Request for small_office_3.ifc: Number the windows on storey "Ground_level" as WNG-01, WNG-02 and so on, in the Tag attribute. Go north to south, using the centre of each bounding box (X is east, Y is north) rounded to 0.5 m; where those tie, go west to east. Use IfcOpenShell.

First a look at what the model holds.

```python
import ifcopenshell
import ifcopenshell.util.element
import ifcopenshell.util.placement

model = ifcopenshell.open("small_office_3.ifc")
print(model.schema)
storey = next(s for s in model.by_type("IfcBuildingStorey") if s.Name == "Ground_level")
windows = [e for e in ifcopenshell.util.element.get_decomposition(storey) if e.is_a("IfcWindow")]
for e in sorted(windows, key=lambda e: e.id()):
    origin = ifcopenshell.util.placement.get_local_placement(e.ObjectPlacement)[:3, 3]
    print(e.id(), e.Tag, e.Name, origin.round(2) + 0.0, sep=" | ")
```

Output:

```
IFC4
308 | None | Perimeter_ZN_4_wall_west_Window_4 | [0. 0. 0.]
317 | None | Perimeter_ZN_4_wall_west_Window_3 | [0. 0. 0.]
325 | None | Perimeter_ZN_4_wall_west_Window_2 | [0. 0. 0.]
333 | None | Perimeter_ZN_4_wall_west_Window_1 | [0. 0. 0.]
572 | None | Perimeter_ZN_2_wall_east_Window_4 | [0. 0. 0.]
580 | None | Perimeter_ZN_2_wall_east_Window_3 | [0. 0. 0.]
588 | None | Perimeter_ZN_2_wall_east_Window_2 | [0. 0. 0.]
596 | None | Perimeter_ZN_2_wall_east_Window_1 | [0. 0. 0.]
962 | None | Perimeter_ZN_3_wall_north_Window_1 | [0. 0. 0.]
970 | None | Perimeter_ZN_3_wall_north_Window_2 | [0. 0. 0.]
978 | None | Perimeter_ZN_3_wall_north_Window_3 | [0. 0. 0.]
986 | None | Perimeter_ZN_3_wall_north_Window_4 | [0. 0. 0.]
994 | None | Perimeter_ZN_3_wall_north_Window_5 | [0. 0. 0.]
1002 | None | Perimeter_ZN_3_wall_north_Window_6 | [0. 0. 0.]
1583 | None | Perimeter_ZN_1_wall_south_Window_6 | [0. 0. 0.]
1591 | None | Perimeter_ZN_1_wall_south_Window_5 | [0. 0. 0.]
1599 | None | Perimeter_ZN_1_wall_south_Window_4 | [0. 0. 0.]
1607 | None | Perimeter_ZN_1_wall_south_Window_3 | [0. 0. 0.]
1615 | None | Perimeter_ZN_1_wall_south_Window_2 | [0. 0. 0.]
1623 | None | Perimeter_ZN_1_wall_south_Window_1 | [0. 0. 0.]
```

```python
import ifcopenshell
import ifcopenshell.geom
import ifcopenshell.util.element
import ifcopenshell.util.shape

model = ifcopenshell.open("small_office_3.ifc")
settings = ifcopenshell.geom.settings()
settings.set("use-world-coords", True)


def centre(element):
    shape = ifcopenshell.geom.create_shape(settings, element)
    return ifcopenshell.util.shape.get_bbox_centroid(shape.geometry)


storey = next(s for s in model.by_type("IfcBuildingStorey") if s.Name == "Ground_level")
windows = [e for e in ifcopenshell.util.element.get_decomposition(storey) if e.is_a("IfcWindow")]

# Insertion points can sit at a corner or the storey origin, so sort by the geometry (in metres).
centres = {e: centre(e) for e in windows}
windows.sort(key=lambda e: (-round(centres[e][1] / 0.5), centres[e][0]))

for i, e in enumerate(windows, start=1):
    number = f"WNG-{i:02d}"
    e.Tag = number
    print(e.id(), number)

model.write("small_office_3_edited.ifc")
```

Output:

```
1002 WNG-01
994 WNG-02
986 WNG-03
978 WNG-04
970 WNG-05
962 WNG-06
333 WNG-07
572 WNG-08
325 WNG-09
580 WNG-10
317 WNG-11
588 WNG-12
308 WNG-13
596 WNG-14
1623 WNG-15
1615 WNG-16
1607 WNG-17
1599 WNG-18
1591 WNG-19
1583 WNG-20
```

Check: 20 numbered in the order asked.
